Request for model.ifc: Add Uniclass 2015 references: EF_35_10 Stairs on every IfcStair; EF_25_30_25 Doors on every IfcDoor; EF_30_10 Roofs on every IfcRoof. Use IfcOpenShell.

First a look at what the model holds.

```python
import ifcopenshell

model = ifcopenshell.open("model.ifc")
print(model.schema)
print("classifications:", [c.Name for c in model.by_type("IfcClassification")])
for ifc_class in ("IfcDoor", "IfcRoof", "IfcStair", "IfcWall", "IfcWindow"):
    print(ifc_class, len(model.by_type(ifc_class)))
```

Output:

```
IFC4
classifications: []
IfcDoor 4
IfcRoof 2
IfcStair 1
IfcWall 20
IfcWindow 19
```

```python
import ifcopenshell
import ifcopenshell.api.classification

model = ifcopenshell.open("model.ifc")

system = ifcopenshell.api.classification.add_classification(model, classification="Uniclass 2015")

codes = {
    "IfcStair": ("EF_35_10", "Stairs"),
    "IfcDoor": ("EF_25_30_25", "Doors"),
    "IfcRoof": ("EF_30_10", "Roofs"),
}
for ifc_class, (code, name) in codes.items():
    products = model.by_type(ifc_class)
    ifcopenshell.api.classification.add_reference(
        model, products=products, classification=system, identification=code, name=name
    )
    print(code, len(products))

model.write("model-out.ifc")
```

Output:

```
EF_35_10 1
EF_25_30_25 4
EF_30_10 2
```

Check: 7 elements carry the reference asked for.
